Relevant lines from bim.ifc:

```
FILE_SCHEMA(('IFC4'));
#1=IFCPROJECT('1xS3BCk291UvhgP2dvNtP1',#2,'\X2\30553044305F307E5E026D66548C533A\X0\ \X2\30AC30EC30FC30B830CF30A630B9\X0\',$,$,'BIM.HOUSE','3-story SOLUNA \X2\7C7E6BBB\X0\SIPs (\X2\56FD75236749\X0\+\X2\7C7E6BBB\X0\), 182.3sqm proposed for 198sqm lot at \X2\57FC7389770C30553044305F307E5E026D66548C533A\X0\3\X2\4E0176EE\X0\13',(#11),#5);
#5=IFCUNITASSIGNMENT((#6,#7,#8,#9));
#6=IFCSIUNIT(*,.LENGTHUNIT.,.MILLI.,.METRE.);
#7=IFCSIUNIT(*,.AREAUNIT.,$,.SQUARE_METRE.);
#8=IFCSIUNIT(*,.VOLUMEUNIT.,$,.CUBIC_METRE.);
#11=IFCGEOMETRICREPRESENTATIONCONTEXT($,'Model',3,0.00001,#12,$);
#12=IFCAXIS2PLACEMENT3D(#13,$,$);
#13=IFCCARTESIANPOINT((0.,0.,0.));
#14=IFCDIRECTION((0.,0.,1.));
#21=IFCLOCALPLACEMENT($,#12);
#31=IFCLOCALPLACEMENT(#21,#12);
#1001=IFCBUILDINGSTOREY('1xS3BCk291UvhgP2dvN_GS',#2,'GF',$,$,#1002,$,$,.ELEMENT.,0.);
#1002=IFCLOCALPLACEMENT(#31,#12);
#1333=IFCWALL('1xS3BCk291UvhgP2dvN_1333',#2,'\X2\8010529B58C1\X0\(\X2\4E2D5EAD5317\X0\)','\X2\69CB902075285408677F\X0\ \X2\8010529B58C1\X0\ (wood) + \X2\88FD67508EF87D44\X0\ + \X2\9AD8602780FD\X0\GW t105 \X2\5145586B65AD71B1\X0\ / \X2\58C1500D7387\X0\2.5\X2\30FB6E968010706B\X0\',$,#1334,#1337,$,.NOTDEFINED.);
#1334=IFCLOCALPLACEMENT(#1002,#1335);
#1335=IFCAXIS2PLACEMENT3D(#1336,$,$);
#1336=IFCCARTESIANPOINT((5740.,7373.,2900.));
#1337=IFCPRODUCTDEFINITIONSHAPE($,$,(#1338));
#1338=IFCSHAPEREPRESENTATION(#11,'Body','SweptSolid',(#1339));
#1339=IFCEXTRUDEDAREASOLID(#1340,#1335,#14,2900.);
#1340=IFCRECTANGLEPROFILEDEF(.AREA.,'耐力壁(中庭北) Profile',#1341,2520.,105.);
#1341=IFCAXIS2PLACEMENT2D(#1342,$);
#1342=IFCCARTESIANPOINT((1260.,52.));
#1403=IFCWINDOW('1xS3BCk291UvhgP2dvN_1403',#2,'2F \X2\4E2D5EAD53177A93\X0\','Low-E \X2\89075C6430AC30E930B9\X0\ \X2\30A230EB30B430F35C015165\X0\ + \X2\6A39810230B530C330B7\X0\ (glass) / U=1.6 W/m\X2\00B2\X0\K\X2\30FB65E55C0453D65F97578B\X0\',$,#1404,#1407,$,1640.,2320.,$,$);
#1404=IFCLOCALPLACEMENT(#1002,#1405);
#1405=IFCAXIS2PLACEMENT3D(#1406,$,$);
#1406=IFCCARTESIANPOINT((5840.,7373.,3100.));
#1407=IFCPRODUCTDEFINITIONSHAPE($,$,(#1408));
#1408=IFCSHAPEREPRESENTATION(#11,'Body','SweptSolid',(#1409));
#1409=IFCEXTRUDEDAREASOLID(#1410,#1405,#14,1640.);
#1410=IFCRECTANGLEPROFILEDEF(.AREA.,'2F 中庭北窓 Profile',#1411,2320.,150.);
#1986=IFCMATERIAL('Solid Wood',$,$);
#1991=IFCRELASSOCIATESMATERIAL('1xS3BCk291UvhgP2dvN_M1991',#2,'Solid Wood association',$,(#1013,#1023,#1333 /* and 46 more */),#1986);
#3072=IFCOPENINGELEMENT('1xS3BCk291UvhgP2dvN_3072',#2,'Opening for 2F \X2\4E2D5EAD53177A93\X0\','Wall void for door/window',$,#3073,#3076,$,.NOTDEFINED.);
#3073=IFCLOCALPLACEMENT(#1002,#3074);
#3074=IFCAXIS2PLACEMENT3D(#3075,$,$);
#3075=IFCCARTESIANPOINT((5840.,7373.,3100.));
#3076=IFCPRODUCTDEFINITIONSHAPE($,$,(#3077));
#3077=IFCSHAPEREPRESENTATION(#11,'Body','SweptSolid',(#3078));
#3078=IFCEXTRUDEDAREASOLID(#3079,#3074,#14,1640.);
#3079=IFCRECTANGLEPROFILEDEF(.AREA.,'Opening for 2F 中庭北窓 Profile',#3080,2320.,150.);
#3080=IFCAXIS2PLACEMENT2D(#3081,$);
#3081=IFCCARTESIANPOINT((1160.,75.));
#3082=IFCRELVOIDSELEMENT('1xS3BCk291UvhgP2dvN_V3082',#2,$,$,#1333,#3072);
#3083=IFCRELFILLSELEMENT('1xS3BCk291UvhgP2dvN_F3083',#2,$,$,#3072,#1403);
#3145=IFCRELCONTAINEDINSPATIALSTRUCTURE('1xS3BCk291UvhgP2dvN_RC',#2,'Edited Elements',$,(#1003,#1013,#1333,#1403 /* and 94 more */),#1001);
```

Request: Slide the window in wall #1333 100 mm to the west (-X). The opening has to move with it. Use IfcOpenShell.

```python
import ifcopenshell
import ifcopenshell.api.geometry
import ifcopenshell.util.placement

model = ifcopenshell.open("bim.ifc")

window = model.by_guid("1xS3BCk291UvhgP2dvN_1403")
opening = window.FillsVoids[0].RelatingOpeningElement
wall = opening.VoidsElements[0].RelatingBuildingElement

wall_matrix = ifcopenshell.util.placement.get_local_placement(wall.ObjectPlacement)
shift = wall_matrix[:3, 0] * -100.0
before = ifcopenshell.util.placement.get_local_placement(window.ObjectPlacement)[:3, 3].copy()

# The window is not placed relative to its opening, so move both.
for product in (opening, window):
    matrix = ifcopenshell.util.placement.get_local_placement(product.ObjectPlacement)
    matrix[:3, 3] += shift
    ifcopenshell.api.geometry.edit_object_placement(model, product=product, matrix=matrix, is_si=False)

after = ifcopenshell.util.placement.get_local_placement(window.ObjectPlacement)[:3, 3]
print("window moved by", (after - before).round(3) + 0.0)

model.write("bim-out.ifc")
```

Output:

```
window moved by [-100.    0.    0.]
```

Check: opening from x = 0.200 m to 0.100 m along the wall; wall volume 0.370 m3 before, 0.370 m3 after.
